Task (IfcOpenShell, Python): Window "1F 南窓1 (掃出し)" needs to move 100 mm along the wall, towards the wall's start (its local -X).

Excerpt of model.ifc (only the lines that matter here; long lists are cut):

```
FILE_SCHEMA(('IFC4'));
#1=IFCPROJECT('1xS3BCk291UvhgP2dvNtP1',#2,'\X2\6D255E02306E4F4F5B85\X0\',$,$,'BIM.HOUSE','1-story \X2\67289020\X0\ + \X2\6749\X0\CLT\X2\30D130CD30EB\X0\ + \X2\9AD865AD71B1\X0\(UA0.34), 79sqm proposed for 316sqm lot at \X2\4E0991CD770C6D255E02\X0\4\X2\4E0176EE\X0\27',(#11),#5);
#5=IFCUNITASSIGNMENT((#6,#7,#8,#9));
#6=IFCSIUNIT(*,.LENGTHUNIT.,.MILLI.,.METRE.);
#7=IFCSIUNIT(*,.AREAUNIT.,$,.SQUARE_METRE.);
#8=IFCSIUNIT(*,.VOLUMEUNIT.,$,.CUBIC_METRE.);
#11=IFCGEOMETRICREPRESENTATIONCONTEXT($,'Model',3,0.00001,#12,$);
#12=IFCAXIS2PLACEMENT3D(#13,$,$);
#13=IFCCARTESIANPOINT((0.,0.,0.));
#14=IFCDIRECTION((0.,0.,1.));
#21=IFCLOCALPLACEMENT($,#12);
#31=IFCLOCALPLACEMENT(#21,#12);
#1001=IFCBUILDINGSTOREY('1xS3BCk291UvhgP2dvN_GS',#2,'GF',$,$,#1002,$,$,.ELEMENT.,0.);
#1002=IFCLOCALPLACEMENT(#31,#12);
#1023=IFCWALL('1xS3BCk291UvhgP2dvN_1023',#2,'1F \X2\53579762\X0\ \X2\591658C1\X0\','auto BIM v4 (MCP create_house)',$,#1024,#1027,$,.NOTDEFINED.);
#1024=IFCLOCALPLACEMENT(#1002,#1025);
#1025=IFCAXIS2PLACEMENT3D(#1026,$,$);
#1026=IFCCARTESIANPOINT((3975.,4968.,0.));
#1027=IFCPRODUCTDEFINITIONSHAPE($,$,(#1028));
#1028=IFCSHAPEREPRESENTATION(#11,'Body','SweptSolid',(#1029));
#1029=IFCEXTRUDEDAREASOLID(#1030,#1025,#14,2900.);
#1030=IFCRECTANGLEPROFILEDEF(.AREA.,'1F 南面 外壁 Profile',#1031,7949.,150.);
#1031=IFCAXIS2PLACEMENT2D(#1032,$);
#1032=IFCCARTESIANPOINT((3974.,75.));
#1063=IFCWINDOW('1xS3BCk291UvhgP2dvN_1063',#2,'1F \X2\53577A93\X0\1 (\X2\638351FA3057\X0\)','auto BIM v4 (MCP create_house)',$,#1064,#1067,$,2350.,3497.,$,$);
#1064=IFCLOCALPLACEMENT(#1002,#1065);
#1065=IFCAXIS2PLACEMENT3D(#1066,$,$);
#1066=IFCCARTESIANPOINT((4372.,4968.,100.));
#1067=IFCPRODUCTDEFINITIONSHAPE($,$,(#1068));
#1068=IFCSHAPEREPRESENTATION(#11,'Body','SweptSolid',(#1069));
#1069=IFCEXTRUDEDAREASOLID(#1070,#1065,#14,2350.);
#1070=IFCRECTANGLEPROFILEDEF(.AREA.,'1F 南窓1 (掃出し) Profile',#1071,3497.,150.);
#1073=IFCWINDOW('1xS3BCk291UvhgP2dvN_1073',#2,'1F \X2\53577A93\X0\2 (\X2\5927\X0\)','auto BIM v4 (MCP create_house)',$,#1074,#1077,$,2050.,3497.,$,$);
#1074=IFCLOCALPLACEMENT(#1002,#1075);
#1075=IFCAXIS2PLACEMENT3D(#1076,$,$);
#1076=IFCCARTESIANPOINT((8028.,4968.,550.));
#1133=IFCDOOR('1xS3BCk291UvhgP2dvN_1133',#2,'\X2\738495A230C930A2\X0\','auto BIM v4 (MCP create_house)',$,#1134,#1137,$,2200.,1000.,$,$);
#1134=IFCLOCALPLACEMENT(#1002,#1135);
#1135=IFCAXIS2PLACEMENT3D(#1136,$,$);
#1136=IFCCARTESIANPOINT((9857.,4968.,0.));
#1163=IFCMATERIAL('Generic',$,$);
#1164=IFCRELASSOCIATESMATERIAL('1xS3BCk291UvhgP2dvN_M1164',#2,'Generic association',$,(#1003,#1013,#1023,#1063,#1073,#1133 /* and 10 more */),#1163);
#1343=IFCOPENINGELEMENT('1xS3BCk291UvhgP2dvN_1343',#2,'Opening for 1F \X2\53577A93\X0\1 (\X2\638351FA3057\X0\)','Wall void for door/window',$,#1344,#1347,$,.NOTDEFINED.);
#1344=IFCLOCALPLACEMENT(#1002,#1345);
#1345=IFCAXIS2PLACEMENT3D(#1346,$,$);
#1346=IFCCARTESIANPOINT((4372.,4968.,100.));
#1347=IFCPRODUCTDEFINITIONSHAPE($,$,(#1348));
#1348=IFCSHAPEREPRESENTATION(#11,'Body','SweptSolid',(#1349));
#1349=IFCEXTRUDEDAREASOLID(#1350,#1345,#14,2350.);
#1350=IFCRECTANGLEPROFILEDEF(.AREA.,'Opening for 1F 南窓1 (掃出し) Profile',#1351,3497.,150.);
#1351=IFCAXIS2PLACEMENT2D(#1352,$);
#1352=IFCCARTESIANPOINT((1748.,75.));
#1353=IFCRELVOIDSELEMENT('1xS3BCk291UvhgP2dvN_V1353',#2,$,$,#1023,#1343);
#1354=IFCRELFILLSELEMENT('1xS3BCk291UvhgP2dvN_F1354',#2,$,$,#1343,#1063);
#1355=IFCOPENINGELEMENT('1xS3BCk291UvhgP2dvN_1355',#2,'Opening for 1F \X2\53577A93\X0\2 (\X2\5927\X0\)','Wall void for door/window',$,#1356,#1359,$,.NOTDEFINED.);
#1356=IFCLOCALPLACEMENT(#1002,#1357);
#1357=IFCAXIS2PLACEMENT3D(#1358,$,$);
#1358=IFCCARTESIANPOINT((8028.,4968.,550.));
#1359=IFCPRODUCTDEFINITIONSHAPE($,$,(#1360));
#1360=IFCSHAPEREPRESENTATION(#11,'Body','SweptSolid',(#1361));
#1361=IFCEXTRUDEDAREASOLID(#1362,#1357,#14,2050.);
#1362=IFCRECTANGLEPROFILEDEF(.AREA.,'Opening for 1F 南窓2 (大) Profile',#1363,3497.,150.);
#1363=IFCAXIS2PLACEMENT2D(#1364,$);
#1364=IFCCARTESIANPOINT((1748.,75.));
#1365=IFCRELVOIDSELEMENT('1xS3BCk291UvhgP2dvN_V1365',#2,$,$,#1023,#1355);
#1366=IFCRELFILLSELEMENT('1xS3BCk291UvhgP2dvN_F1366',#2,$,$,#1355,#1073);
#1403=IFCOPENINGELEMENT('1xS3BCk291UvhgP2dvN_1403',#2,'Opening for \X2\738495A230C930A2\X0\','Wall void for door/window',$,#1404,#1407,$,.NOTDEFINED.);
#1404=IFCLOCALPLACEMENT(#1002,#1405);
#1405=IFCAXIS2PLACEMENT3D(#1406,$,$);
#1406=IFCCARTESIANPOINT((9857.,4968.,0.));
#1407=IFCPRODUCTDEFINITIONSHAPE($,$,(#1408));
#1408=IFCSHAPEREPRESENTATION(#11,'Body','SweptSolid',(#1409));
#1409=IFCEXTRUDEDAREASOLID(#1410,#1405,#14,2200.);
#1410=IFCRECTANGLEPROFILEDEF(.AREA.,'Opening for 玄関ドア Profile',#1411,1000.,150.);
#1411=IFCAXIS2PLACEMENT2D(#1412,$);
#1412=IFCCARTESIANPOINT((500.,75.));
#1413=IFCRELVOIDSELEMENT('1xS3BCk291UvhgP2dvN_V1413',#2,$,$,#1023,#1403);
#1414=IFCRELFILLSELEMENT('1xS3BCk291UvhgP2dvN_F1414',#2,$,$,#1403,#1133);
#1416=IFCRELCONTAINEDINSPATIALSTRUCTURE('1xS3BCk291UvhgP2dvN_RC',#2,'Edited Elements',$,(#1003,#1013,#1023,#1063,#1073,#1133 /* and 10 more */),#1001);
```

```python
import ifcopenshell
import ifcopenshell.api.geometry
import ifcopenshell.util.placement

model = ifcopenshell.open("model.ifc")

window = model.by_guid("1xS3BCk291UvhgP2dvN_1063")
opening = window.FillsVoids[0].RelatingOpeningElement
wall = opening.VoidsElements[0].RelatingBuildingElement

wall_matrix = ifcopenshell.util.placement.get_local_placement(wall.ObjectPlacement)
shift = wall_matrix[:3, 0] * -100.0
before = ifcopenshell.util.placement.get_local_placement(window.ObjectPlacement)[:3, 3].copy()

# The window is not placed relative to its opening, so move both.
for product in (opening, window):
    matrix = ifcopenshell.util.placement.get_local_placement(product.ObjectPlacement)
    matrix[:3, 3] += shift
    ifcopenshell.api.geometry.edit_object_placement(model, product=product, matrix=matrix, is_si=False)

after = ifcopenshell.util.placement.get_local_placement(window.ObjectPlacement)[:3, 3]
print("window moved by", (after - before).round(3) + 0.0)

model.write("model_edited.ifc")
```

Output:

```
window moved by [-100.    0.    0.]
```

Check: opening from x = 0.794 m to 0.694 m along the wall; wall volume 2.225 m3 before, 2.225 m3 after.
